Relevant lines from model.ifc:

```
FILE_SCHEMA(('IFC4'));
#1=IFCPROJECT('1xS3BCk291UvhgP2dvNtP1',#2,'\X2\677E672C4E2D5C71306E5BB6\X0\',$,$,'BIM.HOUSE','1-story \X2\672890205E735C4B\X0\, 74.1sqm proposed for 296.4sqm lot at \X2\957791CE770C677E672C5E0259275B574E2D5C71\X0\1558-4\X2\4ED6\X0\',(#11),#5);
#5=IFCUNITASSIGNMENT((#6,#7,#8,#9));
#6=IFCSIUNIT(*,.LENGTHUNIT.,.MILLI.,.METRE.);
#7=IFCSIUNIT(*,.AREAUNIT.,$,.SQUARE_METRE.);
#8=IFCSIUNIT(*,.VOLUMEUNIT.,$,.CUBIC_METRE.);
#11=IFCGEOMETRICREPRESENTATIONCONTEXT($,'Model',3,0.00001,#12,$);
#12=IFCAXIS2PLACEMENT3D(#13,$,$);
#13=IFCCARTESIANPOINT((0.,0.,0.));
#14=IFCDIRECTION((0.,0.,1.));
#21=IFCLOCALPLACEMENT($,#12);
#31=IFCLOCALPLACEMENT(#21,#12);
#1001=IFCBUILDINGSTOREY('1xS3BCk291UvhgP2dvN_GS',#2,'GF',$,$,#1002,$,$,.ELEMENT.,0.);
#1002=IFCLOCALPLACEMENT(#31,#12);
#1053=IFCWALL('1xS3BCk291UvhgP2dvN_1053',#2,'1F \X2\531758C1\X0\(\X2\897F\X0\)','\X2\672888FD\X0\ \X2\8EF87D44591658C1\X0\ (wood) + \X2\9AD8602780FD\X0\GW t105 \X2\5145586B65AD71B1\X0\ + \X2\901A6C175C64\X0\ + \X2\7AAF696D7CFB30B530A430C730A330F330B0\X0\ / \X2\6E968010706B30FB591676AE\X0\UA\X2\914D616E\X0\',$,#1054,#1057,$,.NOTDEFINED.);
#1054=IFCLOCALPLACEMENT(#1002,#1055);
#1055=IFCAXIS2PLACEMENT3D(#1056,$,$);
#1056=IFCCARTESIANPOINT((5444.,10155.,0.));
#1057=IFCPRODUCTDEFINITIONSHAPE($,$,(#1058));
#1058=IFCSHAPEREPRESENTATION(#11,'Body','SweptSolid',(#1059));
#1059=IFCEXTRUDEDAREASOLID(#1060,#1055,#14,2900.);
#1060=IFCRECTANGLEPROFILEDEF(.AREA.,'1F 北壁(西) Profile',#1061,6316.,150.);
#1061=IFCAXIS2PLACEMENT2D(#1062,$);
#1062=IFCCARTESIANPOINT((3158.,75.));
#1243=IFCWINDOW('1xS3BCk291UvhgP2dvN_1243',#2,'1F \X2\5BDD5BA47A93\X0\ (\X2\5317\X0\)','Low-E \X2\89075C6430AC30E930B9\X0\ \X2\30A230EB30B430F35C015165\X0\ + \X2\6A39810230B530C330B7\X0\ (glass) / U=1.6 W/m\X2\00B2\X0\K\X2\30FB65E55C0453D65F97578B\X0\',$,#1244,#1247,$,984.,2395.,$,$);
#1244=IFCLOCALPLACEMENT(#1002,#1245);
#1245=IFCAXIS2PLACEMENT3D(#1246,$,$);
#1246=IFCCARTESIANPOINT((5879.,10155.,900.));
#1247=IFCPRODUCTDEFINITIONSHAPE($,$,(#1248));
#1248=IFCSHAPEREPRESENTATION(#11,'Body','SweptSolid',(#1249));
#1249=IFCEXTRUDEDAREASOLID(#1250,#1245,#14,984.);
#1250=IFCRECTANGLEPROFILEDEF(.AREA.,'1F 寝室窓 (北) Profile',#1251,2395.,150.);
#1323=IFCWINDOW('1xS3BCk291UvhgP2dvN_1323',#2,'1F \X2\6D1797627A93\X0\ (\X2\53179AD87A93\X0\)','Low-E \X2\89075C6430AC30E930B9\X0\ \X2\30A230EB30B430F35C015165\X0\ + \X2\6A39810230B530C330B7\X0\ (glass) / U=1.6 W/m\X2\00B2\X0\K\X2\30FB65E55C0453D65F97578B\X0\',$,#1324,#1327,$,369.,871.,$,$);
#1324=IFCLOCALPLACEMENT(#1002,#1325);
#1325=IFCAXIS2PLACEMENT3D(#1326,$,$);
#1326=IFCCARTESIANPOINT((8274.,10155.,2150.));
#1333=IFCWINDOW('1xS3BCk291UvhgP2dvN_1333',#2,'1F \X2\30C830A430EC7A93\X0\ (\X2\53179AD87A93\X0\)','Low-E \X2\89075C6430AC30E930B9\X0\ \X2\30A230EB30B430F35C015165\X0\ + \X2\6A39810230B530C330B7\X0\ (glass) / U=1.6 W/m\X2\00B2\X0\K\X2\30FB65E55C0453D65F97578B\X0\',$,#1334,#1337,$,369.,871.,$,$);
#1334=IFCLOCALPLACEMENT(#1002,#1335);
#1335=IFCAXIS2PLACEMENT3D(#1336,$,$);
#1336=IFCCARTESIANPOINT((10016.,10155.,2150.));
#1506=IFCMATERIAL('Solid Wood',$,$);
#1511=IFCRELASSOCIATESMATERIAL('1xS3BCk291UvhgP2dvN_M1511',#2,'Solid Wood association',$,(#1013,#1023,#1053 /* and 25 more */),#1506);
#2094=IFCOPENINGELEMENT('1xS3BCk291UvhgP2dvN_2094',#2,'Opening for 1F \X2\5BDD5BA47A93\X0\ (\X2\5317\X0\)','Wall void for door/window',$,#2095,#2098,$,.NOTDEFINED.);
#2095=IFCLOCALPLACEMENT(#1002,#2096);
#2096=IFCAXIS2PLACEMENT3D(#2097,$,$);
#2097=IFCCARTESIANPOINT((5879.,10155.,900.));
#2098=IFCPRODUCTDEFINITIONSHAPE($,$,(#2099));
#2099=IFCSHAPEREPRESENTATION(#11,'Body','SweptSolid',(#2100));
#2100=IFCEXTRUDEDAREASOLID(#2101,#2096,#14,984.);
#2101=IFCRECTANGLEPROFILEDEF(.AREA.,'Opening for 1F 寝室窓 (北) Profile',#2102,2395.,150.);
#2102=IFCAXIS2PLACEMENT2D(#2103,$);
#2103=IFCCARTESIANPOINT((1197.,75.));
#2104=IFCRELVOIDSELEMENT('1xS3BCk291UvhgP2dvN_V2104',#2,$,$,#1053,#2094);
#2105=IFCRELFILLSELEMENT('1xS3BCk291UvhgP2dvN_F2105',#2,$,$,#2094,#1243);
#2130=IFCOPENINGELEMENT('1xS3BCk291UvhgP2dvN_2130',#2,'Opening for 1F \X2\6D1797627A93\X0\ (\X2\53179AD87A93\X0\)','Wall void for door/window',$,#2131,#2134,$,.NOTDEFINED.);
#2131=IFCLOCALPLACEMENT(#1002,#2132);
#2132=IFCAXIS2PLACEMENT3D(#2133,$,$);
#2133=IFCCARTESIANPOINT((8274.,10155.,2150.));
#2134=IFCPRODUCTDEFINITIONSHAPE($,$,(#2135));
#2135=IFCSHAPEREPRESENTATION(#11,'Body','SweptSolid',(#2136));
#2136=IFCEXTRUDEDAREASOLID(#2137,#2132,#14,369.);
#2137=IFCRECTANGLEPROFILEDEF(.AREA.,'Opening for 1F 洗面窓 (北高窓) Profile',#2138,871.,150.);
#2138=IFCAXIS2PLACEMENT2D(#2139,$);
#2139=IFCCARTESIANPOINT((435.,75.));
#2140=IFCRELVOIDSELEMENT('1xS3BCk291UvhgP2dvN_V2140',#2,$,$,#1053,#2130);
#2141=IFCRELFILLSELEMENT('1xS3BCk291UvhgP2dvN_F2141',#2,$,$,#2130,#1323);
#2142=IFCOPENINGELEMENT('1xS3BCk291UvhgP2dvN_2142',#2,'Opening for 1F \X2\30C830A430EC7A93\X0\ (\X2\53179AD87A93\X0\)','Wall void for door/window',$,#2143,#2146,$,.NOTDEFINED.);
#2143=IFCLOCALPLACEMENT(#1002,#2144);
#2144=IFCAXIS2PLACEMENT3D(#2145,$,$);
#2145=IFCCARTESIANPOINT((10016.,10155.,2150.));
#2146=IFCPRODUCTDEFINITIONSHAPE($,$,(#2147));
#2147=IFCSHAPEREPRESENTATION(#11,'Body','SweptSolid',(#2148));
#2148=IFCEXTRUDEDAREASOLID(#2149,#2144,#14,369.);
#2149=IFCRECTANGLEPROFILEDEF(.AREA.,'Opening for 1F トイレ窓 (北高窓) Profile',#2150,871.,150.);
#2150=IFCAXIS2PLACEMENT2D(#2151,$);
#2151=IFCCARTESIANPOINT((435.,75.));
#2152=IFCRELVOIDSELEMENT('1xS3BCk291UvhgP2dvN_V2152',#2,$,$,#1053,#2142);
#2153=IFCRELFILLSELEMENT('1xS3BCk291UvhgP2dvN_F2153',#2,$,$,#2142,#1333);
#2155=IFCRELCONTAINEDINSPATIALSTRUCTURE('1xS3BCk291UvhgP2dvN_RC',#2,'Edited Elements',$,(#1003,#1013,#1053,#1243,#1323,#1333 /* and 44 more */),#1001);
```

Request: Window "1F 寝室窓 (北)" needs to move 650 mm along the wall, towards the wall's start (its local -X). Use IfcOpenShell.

```python
import ifcopenshell
import ifcopenshell.api.geometry
import ifcopenshell.util.placement
import ifcopenshell.util.unit

model = ifcopenshell.open("model.ifc")
unit_scale = ifcopenshell.util.unit.calculate_unit_scale(model)

window = model.by_guid("1xS3BCk291UvhgP2dvN_1243")
opening = window.FillsVoids[0].RelatingOpeningElement
wall = opening.VoidsElements[0].RelatingBuildingElement

wall_matrix = ifcopenshell.util.placement.get_local_placement(wall.ObjectPlacement)
shift = wall_matrix[:3, 0] * -0.65 / unit_scale
before = ifcopenshell.util.placement.get_local_placement(window.ObjectPlacement)[:3, 3].copy()

# The window is not placed relative to its opening, so move both.
for product in (opening, window):
    matrix = ifcopenshell.util.placement.get_local_placement(product.ObjectPlacement)
    matrix[:3, 3] += shift
    ifcopenshell.api.geometry.edit_object_placement(model, product=product, matrix=matrix, is_si=False)

after = ifcopenshell.util.placement.get_local_placement(window.ObjectPlacement)[:3, 3]
print("window moved by", (after - before).round(3) + 0.0)

model.write("model_rev.ifc")
```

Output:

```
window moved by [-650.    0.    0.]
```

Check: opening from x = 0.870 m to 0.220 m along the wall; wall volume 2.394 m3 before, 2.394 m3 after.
